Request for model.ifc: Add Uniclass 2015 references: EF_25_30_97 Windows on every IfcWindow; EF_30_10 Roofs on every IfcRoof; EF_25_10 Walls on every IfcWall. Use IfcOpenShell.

First a look at what the model holds.

```python
import ifcopenshell

model = ifcopenshell.open("model.ifc")
print(model.schema)
print("classifications:", [c.Name for c in model.by_type("IfcClassification")])
for ifc_class in ("IfcDoor", "IfcRoof", "IfcStair", "IfcWall", "IfcWindow"):
    print(ifc_class, len(model.by_type(ifc_class)))
```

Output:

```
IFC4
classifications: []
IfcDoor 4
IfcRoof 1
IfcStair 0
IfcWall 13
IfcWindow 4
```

```python
import ifcopenshell
import ifcopenshell.api.classification

model = ifcopenshell.open("model.ifc")

system = ifcopenshell.api.classification.add_classification(model, classification="Uniclass 2015")

codes = {
    "IfcWindow": ("EF_25_30_97", "Windows"),
    "IfcRoof": ("EF_30_10", "Roofs"),
    "IfcWall": ("EF_25_10", "Walls"),
}
for ifc_class, (code, name) in codes.items():
    products = model.by_type(ifc_class)
    ifcopenshell.api.classification.add_reference(
        model, products=products, classification=system, identification=code, name=name
    )
    print(code, len(products))

model.write("model-out.ifc")
```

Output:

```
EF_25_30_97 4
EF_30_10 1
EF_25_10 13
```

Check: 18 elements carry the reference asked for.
